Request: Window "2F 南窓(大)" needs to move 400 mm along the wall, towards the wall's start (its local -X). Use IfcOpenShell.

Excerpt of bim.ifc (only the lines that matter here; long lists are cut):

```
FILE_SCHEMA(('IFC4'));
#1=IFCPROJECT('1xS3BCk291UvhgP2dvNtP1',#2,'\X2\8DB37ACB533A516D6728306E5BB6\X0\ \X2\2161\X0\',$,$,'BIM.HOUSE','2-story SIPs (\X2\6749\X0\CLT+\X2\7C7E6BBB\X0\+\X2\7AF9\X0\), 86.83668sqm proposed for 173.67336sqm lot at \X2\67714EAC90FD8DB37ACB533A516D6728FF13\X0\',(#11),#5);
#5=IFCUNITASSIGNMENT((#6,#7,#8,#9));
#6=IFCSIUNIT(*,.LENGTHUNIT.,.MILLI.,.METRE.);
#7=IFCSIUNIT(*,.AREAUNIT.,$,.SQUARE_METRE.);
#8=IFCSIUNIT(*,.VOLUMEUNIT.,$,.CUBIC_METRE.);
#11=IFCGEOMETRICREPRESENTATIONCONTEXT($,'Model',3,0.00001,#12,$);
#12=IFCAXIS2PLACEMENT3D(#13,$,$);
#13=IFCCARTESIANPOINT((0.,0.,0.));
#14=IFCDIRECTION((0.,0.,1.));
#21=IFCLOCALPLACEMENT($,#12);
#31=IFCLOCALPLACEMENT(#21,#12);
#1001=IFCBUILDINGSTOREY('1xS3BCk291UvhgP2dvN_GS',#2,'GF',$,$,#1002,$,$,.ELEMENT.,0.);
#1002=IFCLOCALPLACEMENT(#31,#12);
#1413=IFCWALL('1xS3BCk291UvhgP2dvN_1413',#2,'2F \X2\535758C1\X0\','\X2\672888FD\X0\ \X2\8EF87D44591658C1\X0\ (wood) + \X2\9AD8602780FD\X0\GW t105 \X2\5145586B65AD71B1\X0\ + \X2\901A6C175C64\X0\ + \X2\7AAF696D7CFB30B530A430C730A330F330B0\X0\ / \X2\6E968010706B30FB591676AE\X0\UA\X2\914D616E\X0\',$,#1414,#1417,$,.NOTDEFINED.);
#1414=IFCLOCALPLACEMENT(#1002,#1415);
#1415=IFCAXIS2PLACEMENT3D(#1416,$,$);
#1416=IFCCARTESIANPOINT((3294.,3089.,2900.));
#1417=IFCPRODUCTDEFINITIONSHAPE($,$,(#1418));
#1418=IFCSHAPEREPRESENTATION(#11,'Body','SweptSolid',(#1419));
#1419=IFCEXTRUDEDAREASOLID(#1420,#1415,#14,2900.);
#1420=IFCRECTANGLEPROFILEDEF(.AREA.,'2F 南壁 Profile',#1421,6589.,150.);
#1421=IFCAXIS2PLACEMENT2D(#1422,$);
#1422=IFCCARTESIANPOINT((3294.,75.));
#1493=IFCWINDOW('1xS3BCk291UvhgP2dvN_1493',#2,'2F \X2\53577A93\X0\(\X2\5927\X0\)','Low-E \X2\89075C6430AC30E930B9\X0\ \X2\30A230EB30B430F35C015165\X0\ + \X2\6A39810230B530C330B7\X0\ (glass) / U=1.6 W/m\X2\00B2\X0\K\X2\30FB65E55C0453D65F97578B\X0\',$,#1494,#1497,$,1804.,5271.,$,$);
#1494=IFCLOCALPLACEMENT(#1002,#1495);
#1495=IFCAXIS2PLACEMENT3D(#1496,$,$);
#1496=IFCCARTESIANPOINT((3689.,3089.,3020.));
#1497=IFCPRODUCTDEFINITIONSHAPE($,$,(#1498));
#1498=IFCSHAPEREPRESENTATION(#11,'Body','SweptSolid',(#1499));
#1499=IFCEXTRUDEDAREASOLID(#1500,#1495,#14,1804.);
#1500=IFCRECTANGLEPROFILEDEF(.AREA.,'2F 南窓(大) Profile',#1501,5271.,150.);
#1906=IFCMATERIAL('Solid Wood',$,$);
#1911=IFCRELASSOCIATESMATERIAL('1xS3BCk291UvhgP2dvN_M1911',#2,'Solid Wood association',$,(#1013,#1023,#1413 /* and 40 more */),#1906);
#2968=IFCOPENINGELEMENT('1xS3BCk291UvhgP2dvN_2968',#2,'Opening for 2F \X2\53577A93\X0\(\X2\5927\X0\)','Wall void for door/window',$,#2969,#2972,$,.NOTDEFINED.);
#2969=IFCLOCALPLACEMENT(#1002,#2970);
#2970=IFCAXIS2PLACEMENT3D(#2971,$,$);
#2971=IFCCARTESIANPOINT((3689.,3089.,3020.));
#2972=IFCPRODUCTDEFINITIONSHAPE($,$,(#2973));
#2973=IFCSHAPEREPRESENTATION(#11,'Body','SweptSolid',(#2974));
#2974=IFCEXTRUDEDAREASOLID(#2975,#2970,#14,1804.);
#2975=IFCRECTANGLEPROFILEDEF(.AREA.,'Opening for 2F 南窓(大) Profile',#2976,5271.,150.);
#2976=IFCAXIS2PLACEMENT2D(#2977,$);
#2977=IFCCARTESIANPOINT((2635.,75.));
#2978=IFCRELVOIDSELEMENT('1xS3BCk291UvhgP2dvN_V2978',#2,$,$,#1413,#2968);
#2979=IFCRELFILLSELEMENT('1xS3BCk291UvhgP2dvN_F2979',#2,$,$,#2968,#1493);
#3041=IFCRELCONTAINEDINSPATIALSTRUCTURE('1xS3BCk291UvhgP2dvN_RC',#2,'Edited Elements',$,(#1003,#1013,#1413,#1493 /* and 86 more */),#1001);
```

```python
import ifcopenshell
import ifcopenshell.api.geometry
import ifcopenshell.util.placement

model = ifcopenshell.open("bim.ifc")

window = model.by_guid("1xS3BCk291UvhgP2dvN_1493")
opening = window.FillsVoids[0].RelatingOpeningElement
wall = opening.VoidsElements[0].RelatingBuildingElement

wall_matrix = ifcopenshell.util.placement.get_local_placement(wall.ObjectPlacement)
shift = wall_matrix[:3, 0] * -400.0
before = ifcopenshell.util.placement.get_local_placement(window.ObjectPlacement)[:3, 3].copy()

# The window is not placed relative to its opening, so move both.
for product in (opening, window):
    matrix = ifcopenshell.util.placement.get_local_placement(product.ObjectPlacement)
    matrix[:3, 3] += shift
    ifcopenshell.api.geometry.edit_object_placement(model, product=product, matrix=matrix, is_si=False)

after = ifcopenshell.util.placement.get_local_placement(window.ObjectPlacement)[:3, 3]
print("window moved by", (after - before).round(3) + 0.0)

model.write("bim_v2.ifc")
```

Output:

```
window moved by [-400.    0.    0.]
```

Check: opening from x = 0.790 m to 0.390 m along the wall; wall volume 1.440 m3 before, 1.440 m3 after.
